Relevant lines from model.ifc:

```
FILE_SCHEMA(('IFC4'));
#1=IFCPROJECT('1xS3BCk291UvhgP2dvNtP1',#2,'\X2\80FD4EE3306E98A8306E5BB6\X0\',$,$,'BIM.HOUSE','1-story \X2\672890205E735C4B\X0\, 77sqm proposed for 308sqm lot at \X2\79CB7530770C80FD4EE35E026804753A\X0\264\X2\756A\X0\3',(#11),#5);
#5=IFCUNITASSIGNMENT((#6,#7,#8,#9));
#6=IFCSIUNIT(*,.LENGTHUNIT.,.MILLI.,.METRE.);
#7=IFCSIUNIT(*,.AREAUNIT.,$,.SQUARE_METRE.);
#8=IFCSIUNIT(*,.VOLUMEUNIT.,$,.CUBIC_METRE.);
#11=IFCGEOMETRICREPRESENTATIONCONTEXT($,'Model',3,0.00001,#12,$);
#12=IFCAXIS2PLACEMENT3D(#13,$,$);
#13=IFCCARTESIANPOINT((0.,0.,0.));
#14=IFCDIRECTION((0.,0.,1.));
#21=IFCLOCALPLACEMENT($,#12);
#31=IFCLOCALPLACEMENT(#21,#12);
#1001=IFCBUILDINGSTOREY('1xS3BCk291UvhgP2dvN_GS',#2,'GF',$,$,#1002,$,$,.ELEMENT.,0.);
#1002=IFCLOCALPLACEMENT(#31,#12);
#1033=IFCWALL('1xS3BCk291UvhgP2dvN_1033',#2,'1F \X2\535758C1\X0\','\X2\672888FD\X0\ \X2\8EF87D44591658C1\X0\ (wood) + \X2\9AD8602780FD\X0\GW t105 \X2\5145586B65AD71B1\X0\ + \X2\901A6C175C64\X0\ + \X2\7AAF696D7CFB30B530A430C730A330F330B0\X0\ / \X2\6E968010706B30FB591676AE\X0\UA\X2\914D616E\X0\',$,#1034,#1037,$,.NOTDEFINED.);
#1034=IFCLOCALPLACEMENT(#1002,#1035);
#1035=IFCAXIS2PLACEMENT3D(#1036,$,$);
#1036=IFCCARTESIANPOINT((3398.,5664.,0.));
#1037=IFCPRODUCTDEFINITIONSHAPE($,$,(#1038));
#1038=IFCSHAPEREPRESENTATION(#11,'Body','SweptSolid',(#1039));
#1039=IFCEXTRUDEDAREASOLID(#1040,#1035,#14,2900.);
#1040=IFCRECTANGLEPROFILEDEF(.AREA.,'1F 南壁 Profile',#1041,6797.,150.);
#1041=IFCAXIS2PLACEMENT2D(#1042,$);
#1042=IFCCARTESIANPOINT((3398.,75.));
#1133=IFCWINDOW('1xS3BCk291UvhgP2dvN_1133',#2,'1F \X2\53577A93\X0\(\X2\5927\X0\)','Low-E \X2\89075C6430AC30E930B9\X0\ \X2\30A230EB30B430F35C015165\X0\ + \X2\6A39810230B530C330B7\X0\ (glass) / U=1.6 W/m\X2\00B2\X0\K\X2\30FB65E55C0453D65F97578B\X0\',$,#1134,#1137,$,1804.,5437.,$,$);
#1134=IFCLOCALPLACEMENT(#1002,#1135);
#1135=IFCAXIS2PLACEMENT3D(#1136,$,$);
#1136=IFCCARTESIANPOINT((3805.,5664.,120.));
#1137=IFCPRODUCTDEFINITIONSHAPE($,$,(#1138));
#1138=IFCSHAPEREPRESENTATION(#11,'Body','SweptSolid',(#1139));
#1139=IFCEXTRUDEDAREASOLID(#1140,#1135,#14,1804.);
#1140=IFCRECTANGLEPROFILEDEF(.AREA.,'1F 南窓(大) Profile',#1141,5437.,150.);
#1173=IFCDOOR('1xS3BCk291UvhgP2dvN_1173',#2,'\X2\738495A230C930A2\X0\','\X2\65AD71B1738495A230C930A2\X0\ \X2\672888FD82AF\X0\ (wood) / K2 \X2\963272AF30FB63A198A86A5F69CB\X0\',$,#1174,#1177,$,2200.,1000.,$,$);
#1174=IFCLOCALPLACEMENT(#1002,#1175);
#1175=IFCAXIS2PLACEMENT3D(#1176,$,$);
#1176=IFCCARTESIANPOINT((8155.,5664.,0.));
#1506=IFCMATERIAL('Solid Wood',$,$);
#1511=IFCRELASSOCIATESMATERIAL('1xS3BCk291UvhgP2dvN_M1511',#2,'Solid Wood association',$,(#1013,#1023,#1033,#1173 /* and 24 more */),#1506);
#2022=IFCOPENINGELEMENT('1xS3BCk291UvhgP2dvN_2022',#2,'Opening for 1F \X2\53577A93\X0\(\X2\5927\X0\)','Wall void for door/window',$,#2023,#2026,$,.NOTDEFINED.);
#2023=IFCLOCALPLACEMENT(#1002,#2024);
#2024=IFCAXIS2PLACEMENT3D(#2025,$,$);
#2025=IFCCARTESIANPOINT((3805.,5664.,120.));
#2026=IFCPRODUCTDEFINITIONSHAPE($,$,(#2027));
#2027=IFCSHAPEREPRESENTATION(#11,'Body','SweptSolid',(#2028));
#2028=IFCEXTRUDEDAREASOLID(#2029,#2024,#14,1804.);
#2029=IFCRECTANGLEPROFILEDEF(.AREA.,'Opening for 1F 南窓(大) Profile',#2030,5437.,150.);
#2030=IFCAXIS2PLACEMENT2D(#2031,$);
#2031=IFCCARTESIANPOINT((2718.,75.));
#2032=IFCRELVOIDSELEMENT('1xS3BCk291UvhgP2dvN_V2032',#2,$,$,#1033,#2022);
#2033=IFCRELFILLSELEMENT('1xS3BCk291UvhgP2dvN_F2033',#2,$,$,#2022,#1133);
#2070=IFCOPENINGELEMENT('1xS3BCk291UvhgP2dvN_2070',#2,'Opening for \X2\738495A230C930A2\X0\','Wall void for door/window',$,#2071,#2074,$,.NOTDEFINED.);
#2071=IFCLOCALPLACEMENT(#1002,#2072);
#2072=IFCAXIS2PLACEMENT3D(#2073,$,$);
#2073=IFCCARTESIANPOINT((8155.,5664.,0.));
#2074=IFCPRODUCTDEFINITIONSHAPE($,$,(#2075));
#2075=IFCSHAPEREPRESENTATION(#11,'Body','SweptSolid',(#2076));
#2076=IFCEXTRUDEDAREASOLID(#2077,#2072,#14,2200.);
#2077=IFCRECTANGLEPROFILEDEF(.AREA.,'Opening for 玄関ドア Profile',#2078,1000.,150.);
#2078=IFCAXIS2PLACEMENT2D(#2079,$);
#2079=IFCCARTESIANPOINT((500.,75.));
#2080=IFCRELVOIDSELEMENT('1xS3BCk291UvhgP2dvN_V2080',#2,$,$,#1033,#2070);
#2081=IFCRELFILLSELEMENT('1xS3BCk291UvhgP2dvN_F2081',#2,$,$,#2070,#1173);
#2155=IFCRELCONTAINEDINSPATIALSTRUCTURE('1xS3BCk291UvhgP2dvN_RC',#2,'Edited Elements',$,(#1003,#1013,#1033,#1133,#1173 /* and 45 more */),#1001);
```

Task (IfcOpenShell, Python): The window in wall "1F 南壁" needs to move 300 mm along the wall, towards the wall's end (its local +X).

```python
import ifcopenshell
import ifcopenshell.api.geometry
import ifcopenshell.util.placement
import ifcopenshell.util.unit

model = ifcopenshell.open("model.ifc")
unit_scale = ifcopenshell.util.unit.calculate_unit_scale(model)

window = model.by_guid("1xS3BCk291UvhgP2dvN_1133")
opening = window.FillsVoids[0].RelatingOpeningElement
wall = opening.VoidsElements[0].RelatingBuildingElement

wall_matrix = ifcopenshell.util.placement.get_local_placement(wall.ObjectPlacement)
shift = wall_matrix[:3, 0] * 0.3 / unit_scale
before = ifcopenshell.util.placement.get_local_placement(window.ObjectPlacement)[:3, 3].copy()

# The window is not placed relative to its opening, so move both.
for product in (opening, window):
    matrix = ifcopenshell.util.placement.get_local_placement(product.ObjectPlacement)
    matrix[:3, 3] += shift
    ifcopenshell.api.geometry.edit_object_placement(model, product=product, matrix=matrix, is_si=False)

after = ifcopenshell.util.placement.get_local_placement(window.ObjectPlacement)[:3, 3]
print("window moved by", (after - before).round(3) + 0.0)

model.write("model_rev.ifc")
```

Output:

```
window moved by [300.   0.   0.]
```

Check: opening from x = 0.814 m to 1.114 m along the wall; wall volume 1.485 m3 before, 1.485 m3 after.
